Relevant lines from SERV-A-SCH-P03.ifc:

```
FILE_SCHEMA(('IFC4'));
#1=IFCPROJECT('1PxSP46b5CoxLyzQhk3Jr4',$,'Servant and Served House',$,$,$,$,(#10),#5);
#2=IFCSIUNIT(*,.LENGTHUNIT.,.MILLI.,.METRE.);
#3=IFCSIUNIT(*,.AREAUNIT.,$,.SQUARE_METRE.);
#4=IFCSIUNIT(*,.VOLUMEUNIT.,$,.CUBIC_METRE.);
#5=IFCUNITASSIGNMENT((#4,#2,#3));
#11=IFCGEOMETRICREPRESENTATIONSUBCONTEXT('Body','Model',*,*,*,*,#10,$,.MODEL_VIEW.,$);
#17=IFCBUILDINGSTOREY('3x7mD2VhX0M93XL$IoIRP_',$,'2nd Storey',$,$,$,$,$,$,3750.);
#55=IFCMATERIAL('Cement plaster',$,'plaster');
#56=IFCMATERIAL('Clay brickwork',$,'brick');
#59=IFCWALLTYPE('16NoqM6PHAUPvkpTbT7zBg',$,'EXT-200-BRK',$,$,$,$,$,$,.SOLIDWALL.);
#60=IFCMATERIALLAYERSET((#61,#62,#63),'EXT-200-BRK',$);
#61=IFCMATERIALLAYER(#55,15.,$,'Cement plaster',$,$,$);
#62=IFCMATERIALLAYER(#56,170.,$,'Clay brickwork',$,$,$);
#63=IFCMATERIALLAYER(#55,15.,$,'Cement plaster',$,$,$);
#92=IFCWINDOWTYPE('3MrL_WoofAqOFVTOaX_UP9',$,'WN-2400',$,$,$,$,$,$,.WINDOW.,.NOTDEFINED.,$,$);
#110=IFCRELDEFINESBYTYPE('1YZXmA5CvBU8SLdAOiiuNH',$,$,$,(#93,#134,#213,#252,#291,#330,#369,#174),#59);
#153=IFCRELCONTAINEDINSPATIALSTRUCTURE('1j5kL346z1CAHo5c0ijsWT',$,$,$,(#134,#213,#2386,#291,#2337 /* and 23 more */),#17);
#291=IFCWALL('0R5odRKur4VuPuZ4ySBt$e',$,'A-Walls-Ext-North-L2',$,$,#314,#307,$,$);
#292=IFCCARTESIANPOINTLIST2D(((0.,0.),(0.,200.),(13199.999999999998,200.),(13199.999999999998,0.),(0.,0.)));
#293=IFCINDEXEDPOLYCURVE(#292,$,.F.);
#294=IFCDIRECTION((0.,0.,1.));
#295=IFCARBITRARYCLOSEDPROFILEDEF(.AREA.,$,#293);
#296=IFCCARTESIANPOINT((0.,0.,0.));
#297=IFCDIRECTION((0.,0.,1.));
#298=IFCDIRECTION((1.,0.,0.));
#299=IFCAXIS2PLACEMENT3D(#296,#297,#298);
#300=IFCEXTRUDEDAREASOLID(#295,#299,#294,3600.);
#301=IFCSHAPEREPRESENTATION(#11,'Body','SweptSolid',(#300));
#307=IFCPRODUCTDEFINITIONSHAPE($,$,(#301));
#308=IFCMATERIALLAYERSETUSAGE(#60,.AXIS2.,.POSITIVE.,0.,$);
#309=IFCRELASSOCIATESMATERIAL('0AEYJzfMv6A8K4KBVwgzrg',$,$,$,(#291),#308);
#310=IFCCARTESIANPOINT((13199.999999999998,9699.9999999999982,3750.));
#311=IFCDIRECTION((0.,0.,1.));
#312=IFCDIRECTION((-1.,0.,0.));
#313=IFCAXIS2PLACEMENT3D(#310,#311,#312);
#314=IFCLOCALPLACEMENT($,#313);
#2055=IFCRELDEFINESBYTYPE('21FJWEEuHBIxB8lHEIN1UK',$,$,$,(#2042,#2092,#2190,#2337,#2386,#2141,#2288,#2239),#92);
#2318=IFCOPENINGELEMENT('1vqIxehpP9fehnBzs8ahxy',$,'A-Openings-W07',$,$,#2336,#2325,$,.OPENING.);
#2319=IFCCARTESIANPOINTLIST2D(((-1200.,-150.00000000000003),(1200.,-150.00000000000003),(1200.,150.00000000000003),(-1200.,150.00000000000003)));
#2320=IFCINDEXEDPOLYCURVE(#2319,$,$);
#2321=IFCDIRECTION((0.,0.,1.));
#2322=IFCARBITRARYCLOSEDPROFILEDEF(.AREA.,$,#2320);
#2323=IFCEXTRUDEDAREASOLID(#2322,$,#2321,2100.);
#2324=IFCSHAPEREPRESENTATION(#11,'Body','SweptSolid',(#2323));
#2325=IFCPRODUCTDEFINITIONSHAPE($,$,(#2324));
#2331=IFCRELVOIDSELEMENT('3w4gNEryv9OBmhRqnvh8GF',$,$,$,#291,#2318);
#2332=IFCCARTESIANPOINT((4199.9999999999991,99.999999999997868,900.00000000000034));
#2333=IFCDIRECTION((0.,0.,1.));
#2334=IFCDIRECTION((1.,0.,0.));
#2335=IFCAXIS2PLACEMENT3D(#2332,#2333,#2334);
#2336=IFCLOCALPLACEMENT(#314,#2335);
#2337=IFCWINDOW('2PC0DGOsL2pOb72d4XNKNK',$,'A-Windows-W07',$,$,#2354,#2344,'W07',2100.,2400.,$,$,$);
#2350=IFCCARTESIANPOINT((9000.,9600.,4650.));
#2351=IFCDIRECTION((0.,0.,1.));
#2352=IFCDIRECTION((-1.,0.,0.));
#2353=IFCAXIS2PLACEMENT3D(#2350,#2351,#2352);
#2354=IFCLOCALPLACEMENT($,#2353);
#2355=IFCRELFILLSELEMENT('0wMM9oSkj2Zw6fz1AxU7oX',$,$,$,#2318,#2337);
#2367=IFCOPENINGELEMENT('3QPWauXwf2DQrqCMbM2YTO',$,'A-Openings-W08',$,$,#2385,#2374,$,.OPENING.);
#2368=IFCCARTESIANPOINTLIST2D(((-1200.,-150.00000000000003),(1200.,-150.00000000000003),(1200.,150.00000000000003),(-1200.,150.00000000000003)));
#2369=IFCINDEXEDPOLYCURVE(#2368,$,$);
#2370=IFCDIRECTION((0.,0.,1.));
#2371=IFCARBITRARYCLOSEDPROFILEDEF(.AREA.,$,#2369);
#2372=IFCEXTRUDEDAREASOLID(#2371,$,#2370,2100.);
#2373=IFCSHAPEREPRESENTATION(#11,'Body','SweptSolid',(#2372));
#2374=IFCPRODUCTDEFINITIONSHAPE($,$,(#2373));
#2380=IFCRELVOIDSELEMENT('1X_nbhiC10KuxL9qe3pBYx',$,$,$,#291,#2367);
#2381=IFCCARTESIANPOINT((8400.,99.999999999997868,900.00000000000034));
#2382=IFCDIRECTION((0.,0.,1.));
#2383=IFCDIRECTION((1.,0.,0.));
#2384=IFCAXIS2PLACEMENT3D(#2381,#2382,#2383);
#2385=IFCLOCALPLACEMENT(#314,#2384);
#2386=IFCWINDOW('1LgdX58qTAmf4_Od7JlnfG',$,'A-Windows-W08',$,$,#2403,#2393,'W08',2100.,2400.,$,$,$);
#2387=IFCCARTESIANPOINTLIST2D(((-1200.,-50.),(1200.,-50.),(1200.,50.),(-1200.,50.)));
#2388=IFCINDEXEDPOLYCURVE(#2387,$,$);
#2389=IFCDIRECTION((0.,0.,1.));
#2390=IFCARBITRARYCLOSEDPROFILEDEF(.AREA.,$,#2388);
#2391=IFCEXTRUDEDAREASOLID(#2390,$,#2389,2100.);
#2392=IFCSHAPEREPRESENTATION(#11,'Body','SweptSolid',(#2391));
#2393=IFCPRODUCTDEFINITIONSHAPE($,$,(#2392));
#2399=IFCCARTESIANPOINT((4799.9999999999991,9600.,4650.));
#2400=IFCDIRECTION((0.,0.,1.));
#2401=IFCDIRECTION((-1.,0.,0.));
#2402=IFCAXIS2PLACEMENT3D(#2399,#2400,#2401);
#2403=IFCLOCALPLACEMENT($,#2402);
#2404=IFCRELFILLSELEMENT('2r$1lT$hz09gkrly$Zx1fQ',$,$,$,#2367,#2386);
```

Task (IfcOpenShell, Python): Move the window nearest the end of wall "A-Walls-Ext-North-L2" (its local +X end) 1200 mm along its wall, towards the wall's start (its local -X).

```python
import ifcopenshell
import ifcopenshell.api.geometry
import ifcopenshell.util.placement
import ifcopenshell.util.unit

model = ifcopenshell.open("SERV-A-SCH-P03.ifc")
unit_scale = ifcopenshell.util.unit.calculate_unit_scale(model)

window = model.by_guid("1LgdX58qTAmf4_Od7JlnfG")
opening = window.FillsVoids[0].RelatingOpeningElement
wall = opening.VoidsElements[0].RelatingBuildingElement

wall_matrix = ifcopenshell.util.placement.get_local_placement(wall.ObjectPlacement)
shift = wall_matrix[:3, 0] * -1.2 / unit_scale
before = ifcopenshell.util.placement.get_local_placement(window.ObjectPlacement)[:3, 3].copy()

# The window is not placed relative to its opening, so move both.
for product in (opening, window):
    matrix = ifcopenshell.util.placement.get_local_placement(product.ObjectPlacement)
    matrix[:3, 3] += shift
    ifcopenshell.api.geometry.edit_object_placement(model, product=product, matrix=matrix, is_si=False)

after = ifcopenshell.util.placement.get_local_placement(window.ObjectPlacement)[:3, 3]
print("window moved by", (after - before).round(3) + 0.0)

model.write("SERV-A-SCH-P03_v2.ifc")
```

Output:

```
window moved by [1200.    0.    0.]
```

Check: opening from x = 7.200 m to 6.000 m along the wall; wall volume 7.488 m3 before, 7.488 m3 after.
